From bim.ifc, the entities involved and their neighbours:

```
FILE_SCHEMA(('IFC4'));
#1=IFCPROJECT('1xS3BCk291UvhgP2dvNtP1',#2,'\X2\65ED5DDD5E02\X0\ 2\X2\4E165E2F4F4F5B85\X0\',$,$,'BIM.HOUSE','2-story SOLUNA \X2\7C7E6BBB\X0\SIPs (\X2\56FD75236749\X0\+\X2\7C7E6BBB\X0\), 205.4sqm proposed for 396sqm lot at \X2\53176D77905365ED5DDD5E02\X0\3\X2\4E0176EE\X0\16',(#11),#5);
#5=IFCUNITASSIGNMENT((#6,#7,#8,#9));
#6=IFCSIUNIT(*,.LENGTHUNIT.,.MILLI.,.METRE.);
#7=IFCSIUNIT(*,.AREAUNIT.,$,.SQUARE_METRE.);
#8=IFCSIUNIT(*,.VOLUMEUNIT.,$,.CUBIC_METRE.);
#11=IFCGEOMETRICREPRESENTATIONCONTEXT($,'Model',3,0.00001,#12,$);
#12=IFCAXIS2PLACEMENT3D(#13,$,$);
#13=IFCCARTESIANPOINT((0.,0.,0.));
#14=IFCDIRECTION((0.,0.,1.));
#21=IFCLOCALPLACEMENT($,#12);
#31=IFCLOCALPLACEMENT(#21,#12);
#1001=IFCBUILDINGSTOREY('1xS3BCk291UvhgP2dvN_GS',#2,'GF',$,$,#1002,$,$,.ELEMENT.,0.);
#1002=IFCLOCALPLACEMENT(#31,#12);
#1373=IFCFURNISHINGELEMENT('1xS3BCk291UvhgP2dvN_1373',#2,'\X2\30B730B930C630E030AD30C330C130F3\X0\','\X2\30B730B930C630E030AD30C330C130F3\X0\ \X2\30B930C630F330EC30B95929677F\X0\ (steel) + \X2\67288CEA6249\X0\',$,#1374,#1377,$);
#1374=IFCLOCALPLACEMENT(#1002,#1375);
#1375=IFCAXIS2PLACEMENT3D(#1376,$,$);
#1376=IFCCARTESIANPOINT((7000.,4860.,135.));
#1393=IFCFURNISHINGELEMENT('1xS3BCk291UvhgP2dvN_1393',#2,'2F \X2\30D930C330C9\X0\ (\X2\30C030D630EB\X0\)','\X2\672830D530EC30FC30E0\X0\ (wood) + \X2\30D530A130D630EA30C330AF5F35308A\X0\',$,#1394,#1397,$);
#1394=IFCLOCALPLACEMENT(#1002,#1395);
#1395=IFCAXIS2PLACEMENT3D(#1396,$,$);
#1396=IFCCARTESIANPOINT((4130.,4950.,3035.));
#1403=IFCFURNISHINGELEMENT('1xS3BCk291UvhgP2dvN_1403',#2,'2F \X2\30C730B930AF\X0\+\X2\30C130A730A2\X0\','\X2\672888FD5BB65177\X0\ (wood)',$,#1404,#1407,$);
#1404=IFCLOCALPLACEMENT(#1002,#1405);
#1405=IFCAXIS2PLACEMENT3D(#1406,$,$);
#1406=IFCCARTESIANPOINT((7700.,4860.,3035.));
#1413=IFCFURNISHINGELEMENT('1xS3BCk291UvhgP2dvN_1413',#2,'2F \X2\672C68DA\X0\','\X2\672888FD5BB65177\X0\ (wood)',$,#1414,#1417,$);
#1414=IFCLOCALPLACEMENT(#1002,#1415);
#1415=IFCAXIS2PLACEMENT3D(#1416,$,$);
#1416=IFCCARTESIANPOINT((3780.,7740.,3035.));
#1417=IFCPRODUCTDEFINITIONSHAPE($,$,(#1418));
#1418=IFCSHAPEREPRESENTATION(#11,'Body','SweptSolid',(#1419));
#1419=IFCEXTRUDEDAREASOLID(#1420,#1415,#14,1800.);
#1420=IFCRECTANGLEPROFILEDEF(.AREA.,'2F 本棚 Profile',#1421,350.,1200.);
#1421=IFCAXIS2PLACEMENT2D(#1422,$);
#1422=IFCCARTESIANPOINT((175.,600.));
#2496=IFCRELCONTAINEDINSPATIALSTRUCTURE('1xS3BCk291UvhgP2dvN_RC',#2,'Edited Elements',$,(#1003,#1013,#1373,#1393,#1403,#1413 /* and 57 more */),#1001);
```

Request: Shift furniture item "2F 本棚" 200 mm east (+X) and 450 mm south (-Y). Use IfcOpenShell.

```python
import ifcopenshell
import ifcopenshell.api.geometry
import ifcopenshell.util.placement

model = ifcopenshell.open("bim.ifc")

item = model.by_id(1413)
matrix = ifcopenshell.util.placement.get_local_placement(item.ObjectPlacement)
matrix[0, 3] += 200.0
matrix[1, 3] -= 450.0
ifcopenshell.api.geometry.edit_object_placement(model, product=item, matrix=matrix, is_si=False)

print(ifcopenshell.util.placement.get_local_placement(item.ObjectPlacement).round(3) + 0.0)

model.write("bim_edited.ifc")
```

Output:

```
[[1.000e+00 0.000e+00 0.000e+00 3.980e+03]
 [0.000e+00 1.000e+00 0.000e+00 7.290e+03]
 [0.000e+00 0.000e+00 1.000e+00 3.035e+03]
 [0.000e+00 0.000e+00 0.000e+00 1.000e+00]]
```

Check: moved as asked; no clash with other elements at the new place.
